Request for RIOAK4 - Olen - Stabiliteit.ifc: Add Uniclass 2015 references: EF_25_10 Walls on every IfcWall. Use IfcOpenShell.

First a look at what the model holds.

```python
import ifcopenshell

model = ifcopenshell.open("RIOAK4 - Olen - Stabiliteit.ifc")
print(model.schema)
print("classifications:", [c.Name for c in model.by_type("IfcClassification")])
for ifc_class in ("IfcDoor", "IfcRoof", "IfcStair", "IfcWall", "IfcWindow"):
    print(ifc_class, len(model.by_type(ifc_class)))
```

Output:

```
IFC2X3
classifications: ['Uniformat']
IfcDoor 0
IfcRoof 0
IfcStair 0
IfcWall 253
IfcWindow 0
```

```python
import ifcopenshell
import ifcopenshell.api.classification

model = ifcopenshell.open("RIOAK4 - Olen - Stabiliteit.ifc")

# IFC2X3 requires Source and Edition and has no link from the project to the system.
system = model.create_entity("IfcClassification", Source="NBS", Edition="2015", Name="Uniclass 2015")

codes = {
    "IfcWall": ("EF_25_10", "Walls"),
}
for ifc_class, (code, name) in codes.items():
    products = model.by_type(ifc_class)
    ifcopenshell.api.classification.add_reference(
        model, products=products, classification=system, identification=code, name=name
    )
    print(code, len(products))

model.write("RIOAK4 - Olen - Stabiliteit-out.ifc")
```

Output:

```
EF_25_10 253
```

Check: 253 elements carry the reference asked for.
